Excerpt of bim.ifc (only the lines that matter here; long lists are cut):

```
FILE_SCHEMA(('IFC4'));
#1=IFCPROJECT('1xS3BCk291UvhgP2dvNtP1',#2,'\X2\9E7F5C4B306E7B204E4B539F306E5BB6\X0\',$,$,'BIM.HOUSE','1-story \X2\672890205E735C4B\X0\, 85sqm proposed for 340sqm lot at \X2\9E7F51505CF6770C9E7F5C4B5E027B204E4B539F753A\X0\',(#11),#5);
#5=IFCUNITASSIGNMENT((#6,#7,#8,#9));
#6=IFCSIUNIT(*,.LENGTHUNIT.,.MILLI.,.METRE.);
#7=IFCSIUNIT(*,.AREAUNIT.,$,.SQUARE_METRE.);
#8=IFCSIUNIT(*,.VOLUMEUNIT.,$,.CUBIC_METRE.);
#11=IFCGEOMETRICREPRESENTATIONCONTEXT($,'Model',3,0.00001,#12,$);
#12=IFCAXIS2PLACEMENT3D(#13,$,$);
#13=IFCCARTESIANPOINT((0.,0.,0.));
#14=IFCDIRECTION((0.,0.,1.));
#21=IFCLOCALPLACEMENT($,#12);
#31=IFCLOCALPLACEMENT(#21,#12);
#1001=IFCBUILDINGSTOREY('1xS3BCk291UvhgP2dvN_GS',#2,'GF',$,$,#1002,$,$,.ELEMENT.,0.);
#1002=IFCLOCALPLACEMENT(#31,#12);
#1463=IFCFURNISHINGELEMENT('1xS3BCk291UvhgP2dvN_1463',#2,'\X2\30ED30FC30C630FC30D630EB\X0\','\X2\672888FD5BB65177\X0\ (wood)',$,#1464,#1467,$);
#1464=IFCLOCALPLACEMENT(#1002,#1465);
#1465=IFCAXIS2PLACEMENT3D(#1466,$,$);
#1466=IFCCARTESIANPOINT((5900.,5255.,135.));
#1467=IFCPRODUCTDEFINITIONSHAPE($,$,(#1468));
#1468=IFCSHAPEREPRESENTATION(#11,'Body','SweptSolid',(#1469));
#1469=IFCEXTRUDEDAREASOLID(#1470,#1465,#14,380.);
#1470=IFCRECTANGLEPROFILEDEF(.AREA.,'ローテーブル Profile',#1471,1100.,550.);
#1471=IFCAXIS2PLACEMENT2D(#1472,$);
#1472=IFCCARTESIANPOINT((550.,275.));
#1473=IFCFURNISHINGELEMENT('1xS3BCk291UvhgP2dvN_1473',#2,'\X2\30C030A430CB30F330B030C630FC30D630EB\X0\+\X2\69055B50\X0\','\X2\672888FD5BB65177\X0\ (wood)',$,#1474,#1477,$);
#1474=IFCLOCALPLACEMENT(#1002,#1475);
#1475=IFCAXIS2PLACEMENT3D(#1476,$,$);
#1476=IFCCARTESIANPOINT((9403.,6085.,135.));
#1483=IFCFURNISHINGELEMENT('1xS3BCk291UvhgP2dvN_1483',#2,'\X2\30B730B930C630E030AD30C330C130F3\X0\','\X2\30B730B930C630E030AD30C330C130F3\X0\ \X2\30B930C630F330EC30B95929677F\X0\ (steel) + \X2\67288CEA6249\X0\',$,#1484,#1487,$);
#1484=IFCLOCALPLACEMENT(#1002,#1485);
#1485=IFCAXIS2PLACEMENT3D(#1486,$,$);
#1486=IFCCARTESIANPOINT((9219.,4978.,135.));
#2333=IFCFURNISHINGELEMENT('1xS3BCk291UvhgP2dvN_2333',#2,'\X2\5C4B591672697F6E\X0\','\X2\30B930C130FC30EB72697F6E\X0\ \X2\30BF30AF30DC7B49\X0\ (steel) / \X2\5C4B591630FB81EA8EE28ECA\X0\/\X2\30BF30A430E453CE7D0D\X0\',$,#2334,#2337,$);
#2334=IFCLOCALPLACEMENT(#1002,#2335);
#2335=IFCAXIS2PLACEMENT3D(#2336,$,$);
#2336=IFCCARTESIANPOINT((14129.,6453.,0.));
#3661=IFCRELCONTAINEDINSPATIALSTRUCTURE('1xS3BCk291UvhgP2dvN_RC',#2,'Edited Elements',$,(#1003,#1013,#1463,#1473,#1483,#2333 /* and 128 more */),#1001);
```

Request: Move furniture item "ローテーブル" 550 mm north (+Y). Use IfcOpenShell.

```python
import ifcopenshell
import ifcopenshell.api.geometry
import ifcopenshell.util.placement

model = ifcopenshell.open("bim.ifc")

item = model.by_guid("1xS3BCk291UvhgP2dvN_1463")
matrix = ifcopenshell.util.placement.get_local_placement(item.ObjectPlacement)
matrix[1, 3] += 550.0
ifcopenshell.api.geometry.edit_object_placement(model, product=item, matrix=matrix, is_si=False)

print(ifcopenshell.util.placement.get_local_placement(item.ObjectPlacement).round(3) + 0.0)

model.write("bim_updated.ifc")
```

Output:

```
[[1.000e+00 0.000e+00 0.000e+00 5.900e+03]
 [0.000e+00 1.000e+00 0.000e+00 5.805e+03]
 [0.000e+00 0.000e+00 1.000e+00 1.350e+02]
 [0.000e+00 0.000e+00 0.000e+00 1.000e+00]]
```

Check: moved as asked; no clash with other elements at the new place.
